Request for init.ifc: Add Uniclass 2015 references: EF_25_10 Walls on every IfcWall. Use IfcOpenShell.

First a look at what the model holds.

```python
import ifcopenshell

model = ifcopenshell.open("init.ifc")
print(model.schema)
print("classifications:", [c.Name for c in model.by_type("IfcClassification")])
for ifc_class in ("IfcDoor", "IfcRoof", "IfcStair", "IfcWall", "IfcWindow"):
    print(ifc_class, len(model.by_type(ifc_class)))
```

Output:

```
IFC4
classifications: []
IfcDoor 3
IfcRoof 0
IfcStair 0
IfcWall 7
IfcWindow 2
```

```python
import ifcopenshell
import ifcopenshell.api.classification

model = ifcopenshell.open("init.ifc")

system = ifcopenshell.api.classification.add_classification(model, classification="Uniclass 2015")

codes = {
    "IfcWall": ("EF_25_10", "Walls"),
}
for ifc_class, (code, name) in codes.items():
    products = model.by_type(ifc_class)
    ifcopenshell.api.classification.add_reference(
        model, products=products, classification=system, identification=code, name=name
    )
    print(code, len(products))

model.write("init_v2.ifc")
```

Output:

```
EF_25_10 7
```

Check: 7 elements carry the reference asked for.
